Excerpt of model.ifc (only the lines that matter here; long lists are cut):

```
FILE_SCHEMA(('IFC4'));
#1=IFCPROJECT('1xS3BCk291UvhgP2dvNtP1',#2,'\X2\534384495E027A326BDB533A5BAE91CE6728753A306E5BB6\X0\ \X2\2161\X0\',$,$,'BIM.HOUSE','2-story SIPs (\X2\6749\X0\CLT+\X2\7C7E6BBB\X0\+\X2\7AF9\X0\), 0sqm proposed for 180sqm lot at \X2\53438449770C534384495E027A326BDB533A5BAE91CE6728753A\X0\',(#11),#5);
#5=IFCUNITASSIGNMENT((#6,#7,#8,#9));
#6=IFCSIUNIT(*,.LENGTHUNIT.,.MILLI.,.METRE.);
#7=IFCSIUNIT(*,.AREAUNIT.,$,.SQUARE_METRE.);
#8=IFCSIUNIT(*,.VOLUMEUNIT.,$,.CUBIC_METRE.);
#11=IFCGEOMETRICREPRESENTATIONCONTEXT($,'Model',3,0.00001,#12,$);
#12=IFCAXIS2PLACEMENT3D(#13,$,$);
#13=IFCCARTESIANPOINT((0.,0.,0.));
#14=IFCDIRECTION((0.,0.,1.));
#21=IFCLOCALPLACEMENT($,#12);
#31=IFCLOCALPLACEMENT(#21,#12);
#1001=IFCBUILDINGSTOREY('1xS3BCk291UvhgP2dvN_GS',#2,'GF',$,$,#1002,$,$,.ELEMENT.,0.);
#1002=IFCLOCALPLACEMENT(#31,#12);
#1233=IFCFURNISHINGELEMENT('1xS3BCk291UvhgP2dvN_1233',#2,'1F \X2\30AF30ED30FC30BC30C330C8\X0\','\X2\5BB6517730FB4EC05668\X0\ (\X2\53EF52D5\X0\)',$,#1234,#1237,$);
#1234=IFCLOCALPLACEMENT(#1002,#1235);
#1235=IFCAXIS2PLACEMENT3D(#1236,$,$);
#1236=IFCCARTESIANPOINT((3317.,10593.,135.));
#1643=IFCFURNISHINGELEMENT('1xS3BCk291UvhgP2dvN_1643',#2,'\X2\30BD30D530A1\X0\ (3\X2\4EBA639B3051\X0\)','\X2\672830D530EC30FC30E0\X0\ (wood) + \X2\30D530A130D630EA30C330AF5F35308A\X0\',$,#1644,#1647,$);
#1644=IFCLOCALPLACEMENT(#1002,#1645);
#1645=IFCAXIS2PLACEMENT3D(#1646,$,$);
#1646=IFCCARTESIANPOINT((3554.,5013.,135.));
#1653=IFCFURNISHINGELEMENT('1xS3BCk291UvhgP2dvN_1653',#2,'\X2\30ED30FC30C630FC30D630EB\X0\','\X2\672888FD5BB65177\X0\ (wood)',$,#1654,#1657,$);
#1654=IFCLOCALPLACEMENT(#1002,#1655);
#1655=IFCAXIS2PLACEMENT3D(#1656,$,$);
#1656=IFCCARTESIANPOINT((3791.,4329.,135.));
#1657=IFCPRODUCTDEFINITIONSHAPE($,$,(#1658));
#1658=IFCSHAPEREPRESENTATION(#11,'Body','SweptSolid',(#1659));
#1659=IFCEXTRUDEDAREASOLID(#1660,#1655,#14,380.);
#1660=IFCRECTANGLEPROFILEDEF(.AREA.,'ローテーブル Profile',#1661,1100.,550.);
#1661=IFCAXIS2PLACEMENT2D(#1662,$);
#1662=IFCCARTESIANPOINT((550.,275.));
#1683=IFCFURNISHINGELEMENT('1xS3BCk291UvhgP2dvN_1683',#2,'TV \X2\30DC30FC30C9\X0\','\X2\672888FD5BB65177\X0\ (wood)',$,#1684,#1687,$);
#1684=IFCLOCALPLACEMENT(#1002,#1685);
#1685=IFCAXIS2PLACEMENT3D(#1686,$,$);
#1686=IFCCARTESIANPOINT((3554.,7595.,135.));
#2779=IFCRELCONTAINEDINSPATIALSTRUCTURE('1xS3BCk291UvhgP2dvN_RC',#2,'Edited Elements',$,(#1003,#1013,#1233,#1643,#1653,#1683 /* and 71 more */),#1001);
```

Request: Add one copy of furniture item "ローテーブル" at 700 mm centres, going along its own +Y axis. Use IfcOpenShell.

```python
import ifcopenshell
import ifcopenshell.api.geometry
import ifcopenshell.api.root
import ifcopenshell.util.element
import ifcopenshell.util.placement
import ifcopenshell.util.unit

model = ifcopenshell.open("model.ifc")
unit_scale = ifcopenshell.util.unit.calculate_unit_scale(model)


def reuse_history(source, copy):
    """copy_class also copies each property set's owner history, people and application; keep the originals."""
    for rel in copy.IsDefinedBy:
        if rel.is_a("IfcRelDefinesByProperties") and (history := rel.RelatingPropertyDefinition.OwnerHistory):
            rel.RelatingPropertyDefinition.OwnerHistory = source.OwnerHistory
            ifcopenshell.util.element.remove_deep2(model, history)


source = model.by_guid("1xS3BCk291UvhgP2dvN_1653")
base = ifcopenshell.util.placement.get_local_placement(source.ObjectPlacement)
step = base[:3, 1] * 0.7 / unit_scale

for i in range(1, 2):
    copy = ifcopenshell.api.root.copy_class(model, product=source)
    copy.Representation = ifcopenshell.util.element.copy_deep(
        model, source.Representation, exclude=["IfcGeometricRepresentationContext", "IfcRepresentationMap"]
    )
    reuse_history(source, copy)
    matrix = base.copy()
    matrix[:3, 3] += i * step
    print("added at", matrix[:3, 3].round(3) + 0.0)
    ifcopenshell.api.geometry.edit_object_placement(model, product=copy, matrix=matrix, is_si=False)

model.write("model_edited.ifc")
```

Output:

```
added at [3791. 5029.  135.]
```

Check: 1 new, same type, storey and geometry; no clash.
